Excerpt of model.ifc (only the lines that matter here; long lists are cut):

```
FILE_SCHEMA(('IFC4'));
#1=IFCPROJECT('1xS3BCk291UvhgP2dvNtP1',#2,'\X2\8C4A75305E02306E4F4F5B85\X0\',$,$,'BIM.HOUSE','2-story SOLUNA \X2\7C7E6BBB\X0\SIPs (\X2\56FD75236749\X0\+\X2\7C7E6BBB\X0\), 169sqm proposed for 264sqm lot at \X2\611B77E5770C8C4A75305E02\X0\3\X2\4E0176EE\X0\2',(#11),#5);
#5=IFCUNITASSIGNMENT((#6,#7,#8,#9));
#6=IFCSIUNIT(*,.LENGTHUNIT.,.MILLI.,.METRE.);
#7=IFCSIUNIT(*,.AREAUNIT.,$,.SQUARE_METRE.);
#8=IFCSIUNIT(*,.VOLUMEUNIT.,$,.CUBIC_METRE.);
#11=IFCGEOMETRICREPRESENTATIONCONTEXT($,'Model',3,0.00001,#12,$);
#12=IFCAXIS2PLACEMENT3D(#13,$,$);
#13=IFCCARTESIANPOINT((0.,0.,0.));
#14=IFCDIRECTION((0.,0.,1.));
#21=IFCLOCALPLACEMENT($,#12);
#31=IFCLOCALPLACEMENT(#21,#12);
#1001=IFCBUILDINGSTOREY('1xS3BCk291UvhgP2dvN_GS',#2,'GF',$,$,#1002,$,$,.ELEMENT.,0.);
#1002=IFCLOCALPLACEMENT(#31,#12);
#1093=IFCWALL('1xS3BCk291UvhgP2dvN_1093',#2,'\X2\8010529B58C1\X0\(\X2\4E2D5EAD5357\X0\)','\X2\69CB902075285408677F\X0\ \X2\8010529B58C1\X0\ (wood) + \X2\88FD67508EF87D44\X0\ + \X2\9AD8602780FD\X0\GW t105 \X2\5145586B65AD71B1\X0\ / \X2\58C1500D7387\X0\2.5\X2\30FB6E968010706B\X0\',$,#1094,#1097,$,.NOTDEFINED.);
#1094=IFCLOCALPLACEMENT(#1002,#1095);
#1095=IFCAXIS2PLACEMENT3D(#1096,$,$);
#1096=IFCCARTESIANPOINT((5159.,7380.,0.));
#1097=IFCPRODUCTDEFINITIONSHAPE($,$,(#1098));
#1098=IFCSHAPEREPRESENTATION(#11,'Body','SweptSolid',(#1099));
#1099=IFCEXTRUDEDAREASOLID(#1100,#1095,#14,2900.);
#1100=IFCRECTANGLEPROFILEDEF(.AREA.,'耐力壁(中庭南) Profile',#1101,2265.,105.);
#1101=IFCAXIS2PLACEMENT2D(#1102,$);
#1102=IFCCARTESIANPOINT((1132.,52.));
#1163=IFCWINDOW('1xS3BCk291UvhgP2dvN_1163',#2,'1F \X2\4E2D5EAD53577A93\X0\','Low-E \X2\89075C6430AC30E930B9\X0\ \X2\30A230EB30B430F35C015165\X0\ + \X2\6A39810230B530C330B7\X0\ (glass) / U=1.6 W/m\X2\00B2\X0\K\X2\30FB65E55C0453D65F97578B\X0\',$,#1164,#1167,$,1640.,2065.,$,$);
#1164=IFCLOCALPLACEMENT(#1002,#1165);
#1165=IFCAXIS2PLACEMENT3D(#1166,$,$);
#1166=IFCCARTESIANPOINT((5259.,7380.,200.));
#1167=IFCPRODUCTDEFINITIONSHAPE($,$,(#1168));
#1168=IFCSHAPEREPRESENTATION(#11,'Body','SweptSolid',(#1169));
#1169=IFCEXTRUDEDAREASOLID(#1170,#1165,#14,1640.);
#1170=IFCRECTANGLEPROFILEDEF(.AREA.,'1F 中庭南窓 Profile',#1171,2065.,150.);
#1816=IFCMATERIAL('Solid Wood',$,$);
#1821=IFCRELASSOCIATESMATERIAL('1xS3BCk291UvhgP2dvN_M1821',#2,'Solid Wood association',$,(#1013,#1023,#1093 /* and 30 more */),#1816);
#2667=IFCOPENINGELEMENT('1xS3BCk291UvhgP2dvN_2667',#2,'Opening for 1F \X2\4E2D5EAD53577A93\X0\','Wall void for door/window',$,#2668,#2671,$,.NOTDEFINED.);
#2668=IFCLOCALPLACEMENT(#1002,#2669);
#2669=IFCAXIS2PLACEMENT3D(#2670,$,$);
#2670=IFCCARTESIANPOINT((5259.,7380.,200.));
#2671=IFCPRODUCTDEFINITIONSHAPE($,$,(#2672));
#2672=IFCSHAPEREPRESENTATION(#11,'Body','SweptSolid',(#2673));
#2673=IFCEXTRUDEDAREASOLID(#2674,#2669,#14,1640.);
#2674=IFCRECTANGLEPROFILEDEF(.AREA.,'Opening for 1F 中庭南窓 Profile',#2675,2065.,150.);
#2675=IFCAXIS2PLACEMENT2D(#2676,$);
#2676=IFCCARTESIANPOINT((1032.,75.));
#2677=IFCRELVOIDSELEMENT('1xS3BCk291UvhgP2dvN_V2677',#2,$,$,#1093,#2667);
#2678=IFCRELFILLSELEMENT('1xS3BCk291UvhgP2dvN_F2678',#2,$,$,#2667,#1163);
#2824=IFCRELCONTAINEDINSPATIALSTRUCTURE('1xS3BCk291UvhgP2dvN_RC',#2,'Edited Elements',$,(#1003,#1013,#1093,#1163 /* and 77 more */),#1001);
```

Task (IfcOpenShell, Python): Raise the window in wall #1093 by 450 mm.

```python
import numpy as np
import ifcopenshell
import ifcopenshell.api.geometry
import ifcopenshell.util.placement
import ifcopenshell.util.unit

model = ifcopenshell.open("model.ifc")
unit_scale = ifcopenshell.util.unit.calculate_unit_scale(model)

window = model.by_guid("1xS3BCk291UvhgP2dvN_1163")
opening = window.FillsVoids[0].RelatingOpeningElement
dz = 0.45 / unit_scale

shift = np.array([0.0, 0.0, dz])
# The window is not placed relative to its opening, so move both.
for product in (opening, window):
    matrix = ifcopenshell.util.placement.get_local_placement(product.ObjectPlacement)
    matrix[:3, 3] += shift
    ifcopenshell.api.geometry.edit_object_placement(model, product=product, matrix=matrix, is_si=False)

print(f"moved by {dz * unit_scale:+.3f} m")

model.write("model_edited.ifc")
```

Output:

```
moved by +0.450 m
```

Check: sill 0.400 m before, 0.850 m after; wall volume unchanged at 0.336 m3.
